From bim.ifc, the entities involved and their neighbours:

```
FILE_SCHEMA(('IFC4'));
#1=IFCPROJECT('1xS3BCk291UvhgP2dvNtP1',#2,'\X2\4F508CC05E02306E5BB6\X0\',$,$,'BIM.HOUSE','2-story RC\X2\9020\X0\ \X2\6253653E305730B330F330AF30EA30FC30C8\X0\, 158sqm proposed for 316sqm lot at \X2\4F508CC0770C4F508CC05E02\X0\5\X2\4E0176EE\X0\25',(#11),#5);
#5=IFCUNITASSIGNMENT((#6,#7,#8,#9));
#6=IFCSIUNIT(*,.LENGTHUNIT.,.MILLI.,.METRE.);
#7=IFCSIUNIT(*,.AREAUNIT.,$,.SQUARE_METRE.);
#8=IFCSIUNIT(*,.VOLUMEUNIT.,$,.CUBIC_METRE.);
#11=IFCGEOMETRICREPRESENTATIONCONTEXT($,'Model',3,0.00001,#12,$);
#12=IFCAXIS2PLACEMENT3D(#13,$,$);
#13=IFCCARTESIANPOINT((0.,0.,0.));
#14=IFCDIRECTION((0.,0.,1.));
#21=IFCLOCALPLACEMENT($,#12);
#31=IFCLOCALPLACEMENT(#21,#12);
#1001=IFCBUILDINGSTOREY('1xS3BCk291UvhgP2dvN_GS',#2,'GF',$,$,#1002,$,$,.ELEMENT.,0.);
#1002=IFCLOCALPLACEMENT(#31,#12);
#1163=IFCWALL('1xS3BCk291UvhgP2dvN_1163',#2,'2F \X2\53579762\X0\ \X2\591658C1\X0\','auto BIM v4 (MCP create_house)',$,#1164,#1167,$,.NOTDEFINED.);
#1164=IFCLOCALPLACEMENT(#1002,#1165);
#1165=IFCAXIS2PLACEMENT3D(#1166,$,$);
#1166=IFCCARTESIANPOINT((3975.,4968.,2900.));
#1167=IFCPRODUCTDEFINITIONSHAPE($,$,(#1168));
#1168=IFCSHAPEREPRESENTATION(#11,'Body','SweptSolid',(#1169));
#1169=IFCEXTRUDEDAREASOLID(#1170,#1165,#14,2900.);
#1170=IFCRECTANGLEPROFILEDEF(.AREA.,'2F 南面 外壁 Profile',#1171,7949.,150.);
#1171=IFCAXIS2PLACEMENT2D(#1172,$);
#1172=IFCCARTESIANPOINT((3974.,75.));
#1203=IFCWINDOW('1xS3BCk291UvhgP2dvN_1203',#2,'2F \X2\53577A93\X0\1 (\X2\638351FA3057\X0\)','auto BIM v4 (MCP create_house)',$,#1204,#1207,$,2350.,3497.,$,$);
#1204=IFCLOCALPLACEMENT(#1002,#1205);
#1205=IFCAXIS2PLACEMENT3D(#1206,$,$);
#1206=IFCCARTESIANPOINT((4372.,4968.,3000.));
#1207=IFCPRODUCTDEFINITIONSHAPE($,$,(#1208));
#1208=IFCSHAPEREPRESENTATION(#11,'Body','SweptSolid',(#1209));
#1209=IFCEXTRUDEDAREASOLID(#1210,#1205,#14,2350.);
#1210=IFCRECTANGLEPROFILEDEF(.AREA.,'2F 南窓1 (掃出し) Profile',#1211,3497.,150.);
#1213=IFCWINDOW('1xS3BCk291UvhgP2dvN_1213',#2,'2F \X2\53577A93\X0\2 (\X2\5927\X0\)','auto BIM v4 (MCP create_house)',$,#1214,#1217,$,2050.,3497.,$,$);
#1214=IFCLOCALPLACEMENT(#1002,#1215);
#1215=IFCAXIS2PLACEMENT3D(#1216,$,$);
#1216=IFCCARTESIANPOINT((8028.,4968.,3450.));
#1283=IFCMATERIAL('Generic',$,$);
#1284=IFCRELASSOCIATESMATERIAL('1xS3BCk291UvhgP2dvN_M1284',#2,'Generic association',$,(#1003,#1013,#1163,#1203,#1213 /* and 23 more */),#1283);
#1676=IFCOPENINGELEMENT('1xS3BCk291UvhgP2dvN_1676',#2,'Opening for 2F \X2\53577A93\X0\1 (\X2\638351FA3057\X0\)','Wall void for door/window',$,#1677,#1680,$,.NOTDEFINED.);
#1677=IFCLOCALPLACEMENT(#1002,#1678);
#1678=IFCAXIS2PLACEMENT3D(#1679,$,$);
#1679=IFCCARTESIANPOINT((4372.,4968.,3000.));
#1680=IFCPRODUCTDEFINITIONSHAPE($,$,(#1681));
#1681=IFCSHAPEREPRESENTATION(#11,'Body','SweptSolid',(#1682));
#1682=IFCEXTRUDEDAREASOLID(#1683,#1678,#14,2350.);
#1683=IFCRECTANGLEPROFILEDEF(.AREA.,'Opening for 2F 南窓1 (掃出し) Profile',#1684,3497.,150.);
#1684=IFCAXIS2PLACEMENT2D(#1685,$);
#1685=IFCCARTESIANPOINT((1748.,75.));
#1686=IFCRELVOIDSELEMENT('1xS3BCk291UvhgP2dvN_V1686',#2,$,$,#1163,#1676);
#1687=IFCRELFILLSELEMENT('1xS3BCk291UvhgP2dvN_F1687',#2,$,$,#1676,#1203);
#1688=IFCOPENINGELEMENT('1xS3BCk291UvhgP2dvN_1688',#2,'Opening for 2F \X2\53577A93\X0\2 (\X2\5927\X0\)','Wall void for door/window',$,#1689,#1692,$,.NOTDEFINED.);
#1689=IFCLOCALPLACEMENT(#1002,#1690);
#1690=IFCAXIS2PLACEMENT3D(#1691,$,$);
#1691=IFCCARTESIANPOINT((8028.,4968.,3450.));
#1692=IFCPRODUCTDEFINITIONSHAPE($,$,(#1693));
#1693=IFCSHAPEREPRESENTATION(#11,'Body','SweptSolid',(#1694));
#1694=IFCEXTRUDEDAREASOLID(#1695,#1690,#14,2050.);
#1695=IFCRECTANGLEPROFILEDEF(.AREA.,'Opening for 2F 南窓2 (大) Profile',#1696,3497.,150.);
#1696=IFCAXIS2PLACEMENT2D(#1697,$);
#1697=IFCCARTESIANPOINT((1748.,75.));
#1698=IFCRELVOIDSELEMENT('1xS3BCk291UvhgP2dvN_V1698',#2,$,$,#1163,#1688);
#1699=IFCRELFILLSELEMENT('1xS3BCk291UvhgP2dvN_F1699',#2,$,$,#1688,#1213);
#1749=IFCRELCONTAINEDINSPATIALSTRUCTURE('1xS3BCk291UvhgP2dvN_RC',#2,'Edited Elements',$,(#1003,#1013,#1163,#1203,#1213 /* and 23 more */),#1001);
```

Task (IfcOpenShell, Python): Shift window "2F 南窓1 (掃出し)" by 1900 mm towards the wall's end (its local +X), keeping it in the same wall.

```python
import ifcopenshell
import ifcopenshell.api.geometry
import ifcopenshell.util.placement
import ifcopenshell.util.unit

model = ifcopenshell.open("bim.ifc")
unit_scale = ifcopenshell.util.unit.calculate_unit_scale(model)

window = model.by_guid("1xS3BCk291UvhgP2dvN_1203")
opening = window.FillsVoids[0].RelatingOpeningElement
wall = opening.VoidsElements[0].RelatingBuildingElement

wall_matrix = ifcopenshell.util.placement.get_local_placement(wall.ObjectPlacement)
shift = wall_matrix[:3, 0] * 1.9 / unit_scale
before = ifcopenshell.util.placement.get_local_placement(window.ObjectPlacement)[:3, 3].copy()

# The window is not placed relative to its opening, so move both.
for product in (opening, window):
    matrix = ifcopenshell.util.placement.get_local_placement(product.ObjectPlacement)
    matrix[:3, 3] += shift
    ifcopenshell.api.geometry.edit_object_placement(model, product=product, matrix=matrix, is_si=False)

after = ifcopenshell.util.placement.get_local_placement(window.ObjectPlacement)[:3, 3]
print("window moved by", (after - before).round(3) + 0.0)

model.write("bim_v2.ifc")
```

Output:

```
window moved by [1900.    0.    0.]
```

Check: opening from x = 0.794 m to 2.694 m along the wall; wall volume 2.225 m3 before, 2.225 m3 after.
